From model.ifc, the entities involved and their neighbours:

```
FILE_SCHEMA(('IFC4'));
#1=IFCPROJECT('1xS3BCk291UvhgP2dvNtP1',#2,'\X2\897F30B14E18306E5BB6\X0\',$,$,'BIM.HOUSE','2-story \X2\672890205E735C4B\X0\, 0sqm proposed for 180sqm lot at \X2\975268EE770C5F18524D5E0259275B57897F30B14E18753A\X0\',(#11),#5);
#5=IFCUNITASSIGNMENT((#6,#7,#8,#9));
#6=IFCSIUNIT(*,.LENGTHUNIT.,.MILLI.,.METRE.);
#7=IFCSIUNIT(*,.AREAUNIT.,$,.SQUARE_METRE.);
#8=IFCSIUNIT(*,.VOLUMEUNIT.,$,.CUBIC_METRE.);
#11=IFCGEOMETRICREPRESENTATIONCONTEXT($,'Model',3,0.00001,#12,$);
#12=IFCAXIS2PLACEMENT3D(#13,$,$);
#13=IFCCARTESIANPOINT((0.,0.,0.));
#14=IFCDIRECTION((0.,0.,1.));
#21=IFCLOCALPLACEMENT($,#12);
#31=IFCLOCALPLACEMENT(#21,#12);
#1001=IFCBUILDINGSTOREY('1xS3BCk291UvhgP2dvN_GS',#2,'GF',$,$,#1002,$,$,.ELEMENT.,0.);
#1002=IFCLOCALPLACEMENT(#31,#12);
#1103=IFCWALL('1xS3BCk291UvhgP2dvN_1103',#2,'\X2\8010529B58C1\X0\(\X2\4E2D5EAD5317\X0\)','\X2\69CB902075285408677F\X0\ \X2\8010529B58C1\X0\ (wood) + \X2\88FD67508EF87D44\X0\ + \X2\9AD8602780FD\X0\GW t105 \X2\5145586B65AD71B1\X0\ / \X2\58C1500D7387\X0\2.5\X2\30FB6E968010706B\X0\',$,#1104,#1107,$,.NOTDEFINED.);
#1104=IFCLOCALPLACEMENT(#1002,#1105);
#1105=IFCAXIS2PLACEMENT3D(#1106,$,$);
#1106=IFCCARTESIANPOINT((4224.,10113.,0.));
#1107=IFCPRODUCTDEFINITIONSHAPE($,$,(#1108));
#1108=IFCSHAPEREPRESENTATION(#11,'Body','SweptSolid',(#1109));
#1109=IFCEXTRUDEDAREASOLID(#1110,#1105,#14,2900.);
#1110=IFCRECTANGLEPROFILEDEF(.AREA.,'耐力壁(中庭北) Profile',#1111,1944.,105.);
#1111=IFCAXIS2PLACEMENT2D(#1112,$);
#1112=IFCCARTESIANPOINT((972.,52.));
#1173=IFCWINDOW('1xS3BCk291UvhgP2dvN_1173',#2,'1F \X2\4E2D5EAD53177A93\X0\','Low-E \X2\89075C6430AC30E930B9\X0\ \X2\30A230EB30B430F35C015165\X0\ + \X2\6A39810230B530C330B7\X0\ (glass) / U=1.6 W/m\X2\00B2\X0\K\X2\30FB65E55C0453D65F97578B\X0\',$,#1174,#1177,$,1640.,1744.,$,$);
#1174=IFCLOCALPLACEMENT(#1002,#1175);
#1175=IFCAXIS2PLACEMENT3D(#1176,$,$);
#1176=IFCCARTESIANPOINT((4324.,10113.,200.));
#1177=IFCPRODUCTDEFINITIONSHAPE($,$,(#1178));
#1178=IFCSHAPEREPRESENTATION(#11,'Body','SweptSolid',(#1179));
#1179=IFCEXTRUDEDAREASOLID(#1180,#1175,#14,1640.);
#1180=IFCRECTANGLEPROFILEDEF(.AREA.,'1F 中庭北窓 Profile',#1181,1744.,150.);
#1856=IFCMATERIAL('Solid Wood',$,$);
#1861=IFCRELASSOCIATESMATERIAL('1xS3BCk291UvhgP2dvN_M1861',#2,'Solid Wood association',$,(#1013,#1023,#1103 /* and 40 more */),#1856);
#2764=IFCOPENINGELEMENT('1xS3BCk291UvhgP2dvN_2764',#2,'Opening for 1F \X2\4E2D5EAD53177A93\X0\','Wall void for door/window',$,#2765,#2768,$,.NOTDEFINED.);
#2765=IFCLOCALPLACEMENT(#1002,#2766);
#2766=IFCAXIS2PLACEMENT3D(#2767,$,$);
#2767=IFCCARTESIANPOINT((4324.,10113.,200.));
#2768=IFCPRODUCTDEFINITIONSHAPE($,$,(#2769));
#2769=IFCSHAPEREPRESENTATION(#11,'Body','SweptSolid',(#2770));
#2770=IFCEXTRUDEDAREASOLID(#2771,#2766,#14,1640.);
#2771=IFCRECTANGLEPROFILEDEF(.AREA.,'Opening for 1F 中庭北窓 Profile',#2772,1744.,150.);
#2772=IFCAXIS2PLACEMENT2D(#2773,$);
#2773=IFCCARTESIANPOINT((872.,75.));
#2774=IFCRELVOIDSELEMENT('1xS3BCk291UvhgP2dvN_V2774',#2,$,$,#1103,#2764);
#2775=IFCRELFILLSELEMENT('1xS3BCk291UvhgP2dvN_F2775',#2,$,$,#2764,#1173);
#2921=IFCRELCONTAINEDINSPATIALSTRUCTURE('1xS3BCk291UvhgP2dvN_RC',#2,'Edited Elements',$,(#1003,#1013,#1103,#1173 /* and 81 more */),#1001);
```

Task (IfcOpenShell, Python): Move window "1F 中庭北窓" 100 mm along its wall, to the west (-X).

```python
import ifcopenshell
import ifcopenshell.api.geometry
import ifcopenshell.util.placement
import ifcopenshell.util.unit

model = ifcopenshell.open("model.ifc")
unit_scale = ifcopenshell.util.unit.calculate_unit_scale(model)

window = model.by_guid("1xS3BCk291UvhgP2dvN_1173")
opening = window.FillsVoids[0].RelatingOpeningElement
wall = opening.VoidsElements[0].RelatingBuildingElement

wall_matrix = ifcopenshell.util.placement.get_local_placement(wall.ObjectPlacement)
shift = wall_matrix[:3, 0] * -0.1 / unit_scale
before = ifcopenshell.util.placement.get_local_placement(window.ObjectPlacement)[:3, 3].copy()

# The window is not placed relative to its opening, so move both.
for product in (opening, window):
    matrix = ifcopenshell.util.placement.get_local_placement(product.ObjectPlacement)
    matrix[:3, 3] += shift
    ifcopenshell.api.geometry.edit_object_placement(model, product=product, matrix=matrix, is_si=False)

after = ifcopenshell.util.placement.get_local_placement(window.ObjectPlacement)[:3, 3]
print("window moved by", (after - before).round(3) + 0.0)

model.write("model_v2.ifc")
```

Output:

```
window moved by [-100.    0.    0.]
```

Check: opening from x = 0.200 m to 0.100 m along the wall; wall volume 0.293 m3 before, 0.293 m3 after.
